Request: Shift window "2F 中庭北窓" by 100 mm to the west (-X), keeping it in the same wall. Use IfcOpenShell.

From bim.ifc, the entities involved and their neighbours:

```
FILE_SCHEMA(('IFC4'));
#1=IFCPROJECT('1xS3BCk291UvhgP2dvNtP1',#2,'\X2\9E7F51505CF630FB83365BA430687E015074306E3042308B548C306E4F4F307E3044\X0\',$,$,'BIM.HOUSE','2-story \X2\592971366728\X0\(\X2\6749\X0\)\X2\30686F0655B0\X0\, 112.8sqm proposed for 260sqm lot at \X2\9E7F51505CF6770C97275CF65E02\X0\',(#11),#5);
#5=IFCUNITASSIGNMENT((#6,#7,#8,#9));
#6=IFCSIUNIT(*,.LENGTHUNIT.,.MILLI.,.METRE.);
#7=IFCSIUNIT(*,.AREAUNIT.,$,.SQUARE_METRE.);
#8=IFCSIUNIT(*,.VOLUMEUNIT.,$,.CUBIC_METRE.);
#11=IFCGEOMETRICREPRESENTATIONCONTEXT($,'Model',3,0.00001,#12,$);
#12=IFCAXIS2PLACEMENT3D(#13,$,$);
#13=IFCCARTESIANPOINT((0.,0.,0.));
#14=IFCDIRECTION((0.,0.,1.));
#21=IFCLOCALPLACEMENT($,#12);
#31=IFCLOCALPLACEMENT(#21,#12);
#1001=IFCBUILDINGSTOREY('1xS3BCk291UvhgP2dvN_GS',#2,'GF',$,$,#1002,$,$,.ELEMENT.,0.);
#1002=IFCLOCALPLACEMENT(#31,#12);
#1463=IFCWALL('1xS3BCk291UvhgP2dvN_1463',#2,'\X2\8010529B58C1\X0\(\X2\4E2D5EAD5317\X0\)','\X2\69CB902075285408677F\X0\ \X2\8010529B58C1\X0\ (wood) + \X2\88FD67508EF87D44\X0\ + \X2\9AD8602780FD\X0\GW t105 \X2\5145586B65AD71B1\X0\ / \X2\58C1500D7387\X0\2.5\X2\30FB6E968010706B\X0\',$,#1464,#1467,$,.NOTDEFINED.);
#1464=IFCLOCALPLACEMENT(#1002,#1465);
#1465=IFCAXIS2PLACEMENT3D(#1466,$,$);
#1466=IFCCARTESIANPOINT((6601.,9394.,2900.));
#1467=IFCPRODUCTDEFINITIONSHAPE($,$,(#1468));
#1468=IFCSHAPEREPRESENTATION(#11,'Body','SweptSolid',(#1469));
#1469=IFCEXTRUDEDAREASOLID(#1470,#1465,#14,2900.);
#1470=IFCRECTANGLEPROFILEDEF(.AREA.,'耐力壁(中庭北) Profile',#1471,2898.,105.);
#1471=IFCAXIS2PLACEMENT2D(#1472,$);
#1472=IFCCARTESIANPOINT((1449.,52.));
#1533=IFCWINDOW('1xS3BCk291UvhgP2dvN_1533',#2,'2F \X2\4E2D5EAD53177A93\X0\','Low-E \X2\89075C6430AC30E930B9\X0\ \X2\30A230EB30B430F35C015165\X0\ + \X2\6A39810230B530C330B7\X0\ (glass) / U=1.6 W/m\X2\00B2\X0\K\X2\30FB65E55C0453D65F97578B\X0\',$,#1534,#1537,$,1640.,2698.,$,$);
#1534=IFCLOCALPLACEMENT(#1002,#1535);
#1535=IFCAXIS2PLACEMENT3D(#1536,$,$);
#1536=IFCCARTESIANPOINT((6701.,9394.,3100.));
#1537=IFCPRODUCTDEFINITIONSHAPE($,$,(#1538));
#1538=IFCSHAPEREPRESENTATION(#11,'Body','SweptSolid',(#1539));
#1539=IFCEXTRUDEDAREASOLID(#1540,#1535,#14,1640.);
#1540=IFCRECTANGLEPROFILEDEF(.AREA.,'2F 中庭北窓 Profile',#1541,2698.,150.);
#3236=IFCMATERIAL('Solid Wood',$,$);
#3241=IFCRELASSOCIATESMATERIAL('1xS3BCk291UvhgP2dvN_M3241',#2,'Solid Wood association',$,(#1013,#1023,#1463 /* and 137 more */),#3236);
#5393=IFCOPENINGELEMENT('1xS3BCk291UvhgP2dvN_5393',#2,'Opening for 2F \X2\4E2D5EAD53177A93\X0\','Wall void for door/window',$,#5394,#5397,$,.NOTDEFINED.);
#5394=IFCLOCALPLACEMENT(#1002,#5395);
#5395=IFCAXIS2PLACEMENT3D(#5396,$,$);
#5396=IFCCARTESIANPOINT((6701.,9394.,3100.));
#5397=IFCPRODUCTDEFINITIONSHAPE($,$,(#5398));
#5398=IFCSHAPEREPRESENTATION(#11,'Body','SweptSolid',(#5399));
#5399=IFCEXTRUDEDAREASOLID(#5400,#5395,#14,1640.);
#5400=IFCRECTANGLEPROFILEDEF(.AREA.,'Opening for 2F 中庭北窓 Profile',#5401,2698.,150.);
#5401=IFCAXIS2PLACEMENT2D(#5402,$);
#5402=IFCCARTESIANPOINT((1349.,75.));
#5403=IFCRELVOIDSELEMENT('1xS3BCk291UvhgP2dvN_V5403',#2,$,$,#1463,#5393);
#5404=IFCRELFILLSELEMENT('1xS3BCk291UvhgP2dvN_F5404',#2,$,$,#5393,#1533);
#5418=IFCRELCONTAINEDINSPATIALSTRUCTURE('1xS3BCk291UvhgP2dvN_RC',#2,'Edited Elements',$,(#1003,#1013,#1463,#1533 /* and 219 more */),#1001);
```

```python
import ifcopenshell
import ifcopenshell.api.geometry
import ifcopenshell.util.placement
import ifcopenshell.util.unit

model = ifcopenshell.open("bim.ifc")
unit_scale = ifcopenshell.util.unit.calculate_unit_scale(model)

window = model.by_guid("1xS3BCk291UvhgP2dvN_1533")
opening = window.FillsVoids[0].RelatingOpeningElement
wall = opening.VoidsElements[0].RelatingBuildingElement

wall_matrix = ifcopenshell.util.placement.get_local_placement(wall.ObjectPlacement)
shift = wall_matrix[:3, 0] * -0.1 / unit_scale
before = ifcopenshell.util.placement.get_local_placement(window.ObjectPlacement)[:3, 3].copy()

# The window is not placed relative to its opening, so move both.
for product in (opening, window):
    matrix = ifcopenshell.util.placement.get_local_placement(product.ObjectPlacement)
    matrix[:3, 3] += shift
    ifcopenshell.api.geometry.edit_object_placement(model, product=product, matrix=matrix, is_si=False)

after = ifcopenshell.util.placement.get_local_placement(window.ObjectPlacement)[:3, 3]
print("window moved by", (after - before).round(3) + 0.0)

model.write("bim_updated.ifc")
```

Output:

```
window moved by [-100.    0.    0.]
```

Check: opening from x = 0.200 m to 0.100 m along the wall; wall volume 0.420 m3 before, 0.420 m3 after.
